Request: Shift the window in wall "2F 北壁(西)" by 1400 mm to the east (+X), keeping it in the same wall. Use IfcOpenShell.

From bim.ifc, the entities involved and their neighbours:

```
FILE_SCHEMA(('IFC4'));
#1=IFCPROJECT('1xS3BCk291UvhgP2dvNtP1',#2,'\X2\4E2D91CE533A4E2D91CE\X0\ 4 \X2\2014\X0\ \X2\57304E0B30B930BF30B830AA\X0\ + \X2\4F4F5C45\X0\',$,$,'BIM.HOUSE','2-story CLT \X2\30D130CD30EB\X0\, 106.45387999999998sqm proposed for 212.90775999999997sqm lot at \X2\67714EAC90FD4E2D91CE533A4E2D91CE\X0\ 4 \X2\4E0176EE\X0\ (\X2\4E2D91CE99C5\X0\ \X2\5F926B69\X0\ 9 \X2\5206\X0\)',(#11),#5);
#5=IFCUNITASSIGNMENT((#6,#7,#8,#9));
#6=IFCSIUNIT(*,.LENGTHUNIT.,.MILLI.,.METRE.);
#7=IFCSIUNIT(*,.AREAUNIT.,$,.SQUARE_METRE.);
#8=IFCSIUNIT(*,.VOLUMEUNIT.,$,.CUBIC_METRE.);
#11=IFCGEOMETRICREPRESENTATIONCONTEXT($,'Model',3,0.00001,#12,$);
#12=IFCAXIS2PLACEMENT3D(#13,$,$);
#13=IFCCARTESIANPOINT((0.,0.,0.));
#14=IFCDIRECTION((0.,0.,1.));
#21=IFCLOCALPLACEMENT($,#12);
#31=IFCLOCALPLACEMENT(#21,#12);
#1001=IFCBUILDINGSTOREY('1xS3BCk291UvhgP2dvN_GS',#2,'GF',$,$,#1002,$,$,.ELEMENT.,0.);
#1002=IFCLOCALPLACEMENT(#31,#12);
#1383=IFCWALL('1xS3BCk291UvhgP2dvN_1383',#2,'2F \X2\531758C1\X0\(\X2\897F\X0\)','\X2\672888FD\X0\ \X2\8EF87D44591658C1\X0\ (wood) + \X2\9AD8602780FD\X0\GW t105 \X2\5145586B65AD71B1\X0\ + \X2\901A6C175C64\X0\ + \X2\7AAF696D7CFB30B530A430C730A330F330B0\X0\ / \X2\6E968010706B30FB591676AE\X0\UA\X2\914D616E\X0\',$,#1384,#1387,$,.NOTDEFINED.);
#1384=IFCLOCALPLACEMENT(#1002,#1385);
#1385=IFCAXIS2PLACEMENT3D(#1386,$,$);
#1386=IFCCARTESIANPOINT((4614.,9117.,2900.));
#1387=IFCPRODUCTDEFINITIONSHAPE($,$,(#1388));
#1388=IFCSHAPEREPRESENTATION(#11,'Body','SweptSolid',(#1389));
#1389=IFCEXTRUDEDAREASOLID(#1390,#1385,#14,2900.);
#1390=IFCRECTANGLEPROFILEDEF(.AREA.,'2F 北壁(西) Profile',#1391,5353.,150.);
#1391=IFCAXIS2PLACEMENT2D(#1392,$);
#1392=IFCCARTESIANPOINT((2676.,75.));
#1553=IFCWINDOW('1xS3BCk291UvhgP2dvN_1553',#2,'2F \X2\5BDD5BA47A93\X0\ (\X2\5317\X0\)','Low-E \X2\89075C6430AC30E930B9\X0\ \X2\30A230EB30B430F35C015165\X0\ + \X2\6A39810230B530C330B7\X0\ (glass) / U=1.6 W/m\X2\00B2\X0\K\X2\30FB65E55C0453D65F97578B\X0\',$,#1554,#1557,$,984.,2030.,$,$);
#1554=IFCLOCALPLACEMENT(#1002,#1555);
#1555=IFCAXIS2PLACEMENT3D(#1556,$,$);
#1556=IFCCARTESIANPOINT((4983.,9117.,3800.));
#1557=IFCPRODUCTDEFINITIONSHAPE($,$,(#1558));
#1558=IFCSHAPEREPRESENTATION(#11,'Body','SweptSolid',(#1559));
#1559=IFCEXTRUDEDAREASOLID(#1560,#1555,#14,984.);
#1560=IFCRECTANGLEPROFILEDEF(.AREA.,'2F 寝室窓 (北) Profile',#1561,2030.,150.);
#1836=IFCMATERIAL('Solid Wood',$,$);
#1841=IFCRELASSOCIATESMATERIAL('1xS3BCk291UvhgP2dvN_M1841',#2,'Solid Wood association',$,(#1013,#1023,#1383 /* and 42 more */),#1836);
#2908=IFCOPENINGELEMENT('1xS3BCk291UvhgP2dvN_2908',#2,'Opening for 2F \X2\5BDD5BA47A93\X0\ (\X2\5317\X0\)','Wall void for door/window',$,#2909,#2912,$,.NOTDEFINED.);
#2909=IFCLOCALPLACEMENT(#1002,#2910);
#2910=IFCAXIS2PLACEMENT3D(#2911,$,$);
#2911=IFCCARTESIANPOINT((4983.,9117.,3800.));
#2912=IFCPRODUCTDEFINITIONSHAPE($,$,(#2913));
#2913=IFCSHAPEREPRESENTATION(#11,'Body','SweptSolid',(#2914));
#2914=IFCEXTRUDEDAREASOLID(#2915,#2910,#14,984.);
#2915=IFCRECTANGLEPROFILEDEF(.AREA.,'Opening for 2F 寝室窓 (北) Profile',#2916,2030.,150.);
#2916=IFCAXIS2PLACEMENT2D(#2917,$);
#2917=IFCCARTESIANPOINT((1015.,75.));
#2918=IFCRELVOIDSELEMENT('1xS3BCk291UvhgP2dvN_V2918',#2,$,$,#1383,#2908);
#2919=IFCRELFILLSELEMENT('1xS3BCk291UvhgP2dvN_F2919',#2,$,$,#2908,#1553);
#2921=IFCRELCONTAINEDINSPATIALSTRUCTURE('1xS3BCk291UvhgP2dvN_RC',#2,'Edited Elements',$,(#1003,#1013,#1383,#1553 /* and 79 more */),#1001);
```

```python
import ifcopenshell
import ifcopenshell.api.geometry
import ifcopenshell.util.placement

model = ifcopenshell.open("bim.ifc")

window = model.by_guid("1xS3BCk291UvhgP2dvN_1553")
opening = window.FillsVoids[0].RelatingOpeningElement
wall = opening.VoidsElements[0].RelatingBuildingElement

wall_matrix = ifcopenshell.util.placement.get_local_placement(wall.ObjectPlacement)
shift = wall_matrix[:3, 0] * 1400.0
before = ifcopenshell.util.placement.get_local_placement(window.ObjectPlacement)[:3, 3].copy()

# The window is not placed relative to its opening, so move both.
for product in (opening, window):
    matrix = ifcopenshell.util.placement.get_local_placement(product.ObjectPlacement)
    matrix[:3, 3] += shift
    ifcopenshell.api.geometry.edit_object_placement(model, product=product, matrix=matrix, is_si=False)

after = ifcopenshell.util.placement.get_local_placement(window.ObjectPlacement)[:3, 3]
print("window moved by", (after - before).round(3) + 0.0)

model.write("bim_updated.ifc")
```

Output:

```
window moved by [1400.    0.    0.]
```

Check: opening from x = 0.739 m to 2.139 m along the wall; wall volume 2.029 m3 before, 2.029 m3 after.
